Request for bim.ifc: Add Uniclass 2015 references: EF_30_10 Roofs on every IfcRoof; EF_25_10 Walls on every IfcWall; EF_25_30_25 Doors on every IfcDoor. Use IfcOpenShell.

First a look at what the model holds.

```python
import ifcopenshell

model = ifcopenshell.open("bim.ifc")
print(model.schema)
print("classifications:", [c.Name for c in model.by_type("IfcClassification")])
for ifc_class in ("IfcDoor", "IfcRoof", "IfcStair", "IfcWall", "IfcWindow"):
    print(ifc_class, len(model.by_type(ifc_class)))
```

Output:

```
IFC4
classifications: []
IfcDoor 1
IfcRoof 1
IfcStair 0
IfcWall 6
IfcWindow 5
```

```python
import ifcopenshell
import ifcopenshell.api.classification

model = ifcopenshell.open("bim.ifc")

system = ifcopenshell.api.classification.add_classification(model, classification="Uniclass 2015")

codes = {
    "IfcRoof": ("EF_30_10", "Roofs"),
    "IfcWall": ("EF_25_10", "Walls"),
    "IfcDoor": ("EF_25_30_25", "Doors"),
}
for ifc_class, (code, name) in codes.items():
    products = model.by_type(ifc_class)
    ifcopenshell.api.classification.add_reference(
        model, products=products, classification=system, identification=code, name=name
    )
    print(code, len(products))

model.write("bim_rev.ifc")
```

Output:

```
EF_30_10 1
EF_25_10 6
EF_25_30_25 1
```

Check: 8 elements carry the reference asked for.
